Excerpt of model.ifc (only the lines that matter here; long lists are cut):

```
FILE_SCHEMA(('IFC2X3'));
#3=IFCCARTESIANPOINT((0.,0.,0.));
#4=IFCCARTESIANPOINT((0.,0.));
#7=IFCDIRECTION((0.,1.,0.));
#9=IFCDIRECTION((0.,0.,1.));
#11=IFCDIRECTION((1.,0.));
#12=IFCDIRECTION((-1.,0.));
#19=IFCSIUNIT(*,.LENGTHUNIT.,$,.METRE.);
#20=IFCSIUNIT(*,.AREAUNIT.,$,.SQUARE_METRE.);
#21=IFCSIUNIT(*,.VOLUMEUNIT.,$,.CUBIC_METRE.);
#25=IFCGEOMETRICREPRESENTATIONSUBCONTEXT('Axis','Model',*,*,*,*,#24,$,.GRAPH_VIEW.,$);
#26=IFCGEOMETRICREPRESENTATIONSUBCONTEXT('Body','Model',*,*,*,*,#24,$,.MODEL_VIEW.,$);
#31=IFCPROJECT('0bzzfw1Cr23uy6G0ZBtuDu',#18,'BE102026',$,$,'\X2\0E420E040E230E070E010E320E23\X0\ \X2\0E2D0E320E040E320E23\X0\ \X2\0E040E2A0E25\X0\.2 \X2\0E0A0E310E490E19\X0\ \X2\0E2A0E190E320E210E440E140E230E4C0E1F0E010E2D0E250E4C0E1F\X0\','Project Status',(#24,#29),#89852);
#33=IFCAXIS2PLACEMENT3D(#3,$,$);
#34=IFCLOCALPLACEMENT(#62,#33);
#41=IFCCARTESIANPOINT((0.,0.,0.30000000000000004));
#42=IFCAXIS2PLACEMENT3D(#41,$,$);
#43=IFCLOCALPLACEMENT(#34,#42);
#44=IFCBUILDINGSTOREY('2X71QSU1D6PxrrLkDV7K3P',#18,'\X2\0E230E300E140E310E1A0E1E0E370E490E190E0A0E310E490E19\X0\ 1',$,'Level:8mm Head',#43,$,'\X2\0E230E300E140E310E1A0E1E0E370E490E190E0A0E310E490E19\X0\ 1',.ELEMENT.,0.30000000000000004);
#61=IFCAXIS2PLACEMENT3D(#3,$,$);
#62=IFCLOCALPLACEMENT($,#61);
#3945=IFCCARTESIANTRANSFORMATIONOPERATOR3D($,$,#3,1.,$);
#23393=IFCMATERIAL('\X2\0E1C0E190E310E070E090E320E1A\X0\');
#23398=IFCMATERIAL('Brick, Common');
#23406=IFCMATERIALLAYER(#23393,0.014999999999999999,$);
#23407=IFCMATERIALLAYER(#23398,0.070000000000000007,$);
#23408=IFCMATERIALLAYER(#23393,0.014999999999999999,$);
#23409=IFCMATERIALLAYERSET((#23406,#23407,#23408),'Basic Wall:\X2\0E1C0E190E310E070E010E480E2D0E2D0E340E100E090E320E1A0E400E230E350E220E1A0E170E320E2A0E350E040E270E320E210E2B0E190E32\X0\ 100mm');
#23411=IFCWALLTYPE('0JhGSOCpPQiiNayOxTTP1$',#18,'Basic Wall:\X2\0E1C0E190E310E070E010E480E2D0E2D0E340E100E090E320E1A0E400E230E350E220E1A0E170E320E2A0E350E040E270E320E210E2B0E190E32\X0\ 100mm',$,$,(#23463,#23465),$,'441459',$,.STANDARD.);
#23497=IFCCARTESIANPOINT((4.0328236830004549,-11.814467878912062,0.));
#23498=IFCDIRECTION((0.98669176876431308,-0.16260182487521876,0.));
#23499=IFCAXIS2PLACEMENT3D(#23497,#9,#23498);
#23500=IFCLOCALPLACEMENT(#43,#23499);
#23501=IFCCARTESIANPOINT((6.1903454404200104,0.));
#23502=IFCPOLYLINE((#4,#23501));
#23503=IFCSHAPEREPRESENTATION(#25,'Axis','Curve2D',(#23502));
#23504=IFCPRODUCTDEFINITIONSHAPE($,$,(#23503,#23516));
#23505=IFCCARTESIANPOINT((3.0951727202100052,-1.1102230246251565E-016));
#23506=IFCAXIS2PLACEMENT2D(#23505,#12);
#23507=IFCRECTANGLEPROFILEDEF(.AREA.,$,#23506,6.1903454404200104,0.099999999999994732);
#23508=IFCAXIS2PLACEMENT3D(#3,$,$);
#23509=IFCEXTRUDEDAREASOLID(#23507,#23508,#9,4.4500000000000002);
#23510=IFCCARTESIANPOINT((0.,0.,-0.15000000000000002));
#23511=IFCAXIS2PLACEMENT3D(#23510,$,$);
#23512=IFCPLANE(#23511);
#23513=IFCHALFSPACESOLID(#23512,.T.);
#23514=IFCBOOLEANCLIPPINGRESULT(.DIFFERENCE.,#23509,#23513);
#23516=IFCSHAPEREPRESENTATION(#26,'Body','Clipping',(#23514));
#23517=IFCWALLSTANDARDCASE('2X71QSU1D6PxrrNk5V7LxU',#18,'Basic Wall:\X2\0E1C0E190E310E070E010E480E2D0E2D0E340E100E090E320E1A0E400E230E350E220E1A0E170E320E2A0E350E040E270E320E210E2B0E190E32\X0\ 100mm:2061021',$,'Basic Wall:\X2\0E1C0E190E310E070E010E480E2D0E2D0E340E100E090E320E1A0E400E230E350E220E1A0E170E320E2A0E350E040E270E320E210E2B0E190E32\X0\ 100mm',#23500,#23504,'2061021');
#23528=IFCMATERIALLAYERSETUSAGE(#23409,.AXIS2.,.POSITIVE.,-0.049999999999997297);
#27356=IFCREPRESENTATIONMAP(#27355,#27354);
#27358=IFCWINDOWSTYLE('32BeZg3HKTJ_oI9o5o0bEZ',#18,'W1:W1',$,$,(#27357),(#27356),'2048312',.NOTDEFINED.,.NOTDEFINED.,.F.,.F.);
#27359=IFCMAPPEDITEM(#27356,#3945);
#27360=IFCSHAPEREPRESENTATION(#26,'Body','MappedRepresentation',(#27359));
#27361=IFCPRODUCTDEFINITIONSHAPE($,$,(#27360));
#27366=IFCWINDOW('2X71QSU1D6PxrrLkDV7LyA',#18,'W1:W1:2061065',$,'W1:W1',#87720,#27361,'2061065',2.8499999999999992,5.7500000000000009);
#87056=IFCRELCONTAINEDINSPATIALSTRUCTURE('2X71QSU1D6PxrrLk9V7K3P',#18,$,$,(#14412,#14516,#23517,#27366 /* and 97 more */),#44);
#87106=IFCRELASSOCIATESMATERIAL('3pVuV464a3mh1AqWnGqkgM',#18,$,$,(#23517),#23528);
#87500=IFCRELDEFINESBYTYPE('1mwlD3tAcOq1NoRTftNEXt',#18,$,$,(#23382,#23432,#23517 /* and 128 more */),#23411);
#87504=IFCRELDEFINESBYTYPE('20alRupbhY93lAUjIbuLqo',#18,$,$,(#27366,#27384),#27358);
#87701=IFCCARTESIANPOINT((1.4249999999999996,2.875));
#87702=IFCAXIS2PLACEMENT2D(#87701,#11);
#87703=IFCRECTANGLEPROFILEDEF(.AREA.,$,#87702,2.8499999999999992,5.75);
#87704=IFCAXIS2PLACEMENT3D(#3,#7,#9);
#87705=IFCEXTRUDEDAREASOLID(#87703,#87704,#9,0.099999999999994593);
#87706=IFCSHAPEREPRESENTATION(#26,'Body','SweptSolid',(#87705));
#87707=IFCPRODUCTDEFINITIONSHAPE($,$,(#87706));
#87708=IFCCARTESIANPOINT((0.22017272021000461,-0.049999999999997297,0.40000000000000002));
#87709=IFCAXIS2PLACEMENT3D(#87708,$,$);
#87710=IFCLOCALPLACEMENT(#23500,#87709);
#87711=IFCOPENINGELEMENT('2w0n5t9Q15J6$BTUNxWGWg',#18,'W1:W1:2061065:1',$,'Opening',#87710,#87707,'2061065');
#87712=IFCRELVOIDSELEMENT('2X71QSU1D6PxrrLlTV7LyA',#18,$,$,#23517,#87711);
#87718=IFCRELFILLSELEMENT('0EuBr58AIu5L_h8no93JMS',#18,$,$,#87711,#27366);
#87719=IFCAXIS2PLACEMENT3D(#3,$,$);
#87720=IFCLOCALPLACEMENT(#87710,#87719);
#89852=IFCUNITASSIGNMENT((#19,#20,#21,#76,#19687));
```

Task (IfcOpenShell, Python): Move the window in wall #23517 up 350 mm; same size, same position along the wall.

```python
import numpy as np
import ifcopenshell
import ifcopenshell.api.geometry
import ifcopenshell.util.placement
import ifcopenshell.util.unit

model = ifcopenshell.open("model.ifc")
unit_scale = ifcopenshell.util.unit.calculate_unit_scale(model)

window = model.by_id(27366)
opening = window.FillsVoids[0].RelatingOpeningElement
dz = 0.35

shift = np.array([0.0, 0.0, dz])
# The window is placed relative to its opening, so it follows when the opening moves.
matrix = ifcopenshell.util.placement.get_local_placement(opening.ObjectPlacement)
matrix[:3, 3] += shift
ifcopenshell.api.geometry.edit_object_placement(
    model, product=opening, matrix=matrix, is_si=False, should_transform_children=True
)

print(f"moved by {dz * unit_scale:+.3f} m")

model.write("model_rev.ifc")
```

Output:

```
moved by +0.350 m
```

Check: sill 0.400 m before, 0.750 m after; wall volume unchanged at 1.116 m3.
